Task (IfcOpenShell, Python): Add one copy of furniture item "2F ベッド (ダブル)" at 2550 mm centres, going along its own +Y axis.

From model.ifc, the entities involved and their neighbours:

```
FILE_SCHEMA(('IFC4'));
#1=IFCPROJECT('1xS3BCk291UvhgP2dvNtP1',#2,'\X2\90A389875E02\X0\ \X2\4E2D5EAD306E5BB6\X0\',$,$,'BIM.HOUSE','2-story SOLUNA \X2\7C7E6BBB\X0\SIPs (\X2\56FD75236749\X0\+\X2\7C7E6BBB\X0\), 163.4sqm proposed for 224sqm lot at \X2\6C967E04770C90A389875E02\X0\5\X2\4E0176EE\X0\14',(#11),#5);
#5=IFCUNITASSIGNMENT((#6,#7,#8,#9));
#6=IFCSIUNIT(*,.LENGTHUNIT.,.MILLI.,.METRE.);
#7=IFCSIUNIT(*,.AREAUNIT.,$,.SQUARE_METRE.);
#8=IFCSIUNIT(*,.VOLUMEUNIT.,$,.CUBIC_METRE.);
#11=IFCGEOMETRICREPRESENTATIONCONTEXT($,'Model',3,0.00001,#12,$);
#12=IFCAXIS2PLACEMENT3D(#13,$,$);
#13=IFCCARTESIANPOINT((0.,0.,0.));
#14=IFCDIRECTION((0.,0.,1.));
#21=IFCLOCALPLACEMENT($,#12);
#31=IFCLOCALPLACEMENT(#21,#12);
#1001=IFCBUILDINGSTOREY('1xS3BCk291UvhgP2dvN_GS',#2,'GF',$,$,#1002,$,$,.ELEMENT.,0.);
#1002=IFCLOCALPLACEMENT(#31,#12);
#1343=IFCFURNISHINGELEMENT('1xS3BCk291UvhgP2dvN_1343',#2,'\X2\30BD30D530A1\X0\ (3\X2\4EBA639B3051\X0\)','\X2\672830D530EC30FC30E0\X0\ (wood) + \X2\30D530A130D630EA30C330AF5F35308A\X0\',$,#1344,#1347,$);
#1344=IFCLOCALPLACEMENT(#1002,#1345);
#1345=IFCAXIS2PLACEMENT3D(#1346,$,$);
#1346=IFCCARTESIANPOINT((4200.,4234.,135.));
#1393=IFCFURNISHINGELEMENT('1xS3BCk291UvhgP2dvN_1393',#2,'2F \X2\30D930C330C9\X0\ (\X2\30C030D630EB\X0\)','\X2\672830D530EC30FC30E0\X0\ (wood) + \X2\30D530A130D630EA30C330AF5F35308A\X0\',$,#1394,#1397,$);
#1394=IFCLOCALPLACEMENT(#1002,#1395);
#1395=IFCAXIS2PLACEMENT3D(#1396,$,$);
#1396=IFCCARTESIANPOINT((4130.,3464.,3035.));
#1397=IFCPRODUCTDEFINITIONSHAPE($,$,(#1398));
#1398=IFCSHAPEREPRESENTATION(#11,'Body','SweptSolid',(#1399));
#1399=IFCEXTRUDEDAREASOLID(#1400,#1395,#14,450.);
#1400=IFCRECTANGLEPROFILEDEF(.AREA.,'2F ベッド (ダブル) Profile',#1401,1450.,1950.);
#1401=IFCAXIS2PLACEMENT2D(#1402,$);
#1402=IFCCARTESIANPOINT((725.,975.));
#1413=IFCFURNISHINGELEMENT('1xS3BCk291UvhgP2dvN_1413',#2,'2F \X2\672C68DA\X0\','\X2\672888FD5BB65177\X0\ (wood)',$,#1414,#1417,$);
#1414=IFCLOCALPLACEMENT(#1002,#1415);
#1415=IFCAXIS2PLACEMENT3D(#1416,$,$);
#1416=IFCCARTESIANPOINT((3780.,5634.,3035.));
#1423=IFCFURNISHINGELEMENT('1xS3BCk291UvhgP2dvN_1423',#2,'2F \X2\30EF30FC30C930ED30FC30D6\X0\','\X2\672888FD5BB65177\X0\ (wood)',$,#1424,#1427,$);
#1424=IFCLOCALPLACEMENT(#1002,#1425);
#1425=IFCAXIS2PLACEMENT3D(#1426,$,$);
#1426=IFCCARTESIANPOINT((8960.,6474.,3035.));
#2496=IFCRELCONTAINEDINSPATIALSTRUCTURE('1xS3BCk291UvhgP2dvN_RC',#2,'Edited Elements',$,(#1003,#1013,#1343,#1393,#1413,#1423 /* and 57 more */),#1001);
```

```python
import ifcopenshell
import ifcopenshell.api.geometry
import ifcopenshell.api.root
import ifcopenshell.util.element
import ifcopenshell.util.placement

model = ifcopenshell.open("model.ifc")


def reuse_history(source, copy):
    """copy_class also copies each property set's owner history, people and application; keep the originals."""
    for rel in copy.IsDefinedBy:
        if rel.is_a("IfcRelDefinesByProperties") and (history := rel.RelatingPropertyDefinition.OwnerHistory):
            rel.RelatingPropertyDefinition.OwnerHistory = source.OwnerHistory
            ifcopenshell.util.element.remove_deep2(model, history)


source = model.by_guid("1xS3BCk291UvhgP2dvN_1393")
base = ifcopenshell.util.placement.get_local_placement(source.ObjectPlacement)
step = base[:3, 1] * 2550.0

for i in range(1, 2):
    copy = ifcopenshell.api.root.copy_class(model, product=source)
    copy.Representation = ifcopenshell.util.element.copy_deep(
        model, source.Representation, exclude=["IfcGeometricRepresentationContext", "IfcRepresentationMap"]
    )
    reuse_history(source, copy)
    matrix = base.copy()
    matrix[:3, 3] += i * step
    print("added at", matrix[:3, 3].round(3) + 0.0)
    ifcopenshell.api.geometry.edit_object_placement(model, product=copy, matrix=matrix, is_si=False)

model.write("model_v2.ifc")
```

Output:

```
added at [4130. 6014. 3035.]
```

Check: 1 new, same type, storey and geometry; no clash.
